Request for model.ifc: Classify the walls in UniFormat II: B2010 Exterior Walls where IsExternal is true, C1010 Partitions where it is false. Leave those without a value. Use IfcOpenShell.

First a look at what the model holds.

```python
import ifcopenshell
import ifcopenshell.util.element

model = ifcopenshell.open("model.ifc")
print(model.schema)
print("classifications:", [c.Name for c in model.by_type("IfcClassification")])
values = [ifcopenshell.util.element.get_pset(e, "Pset_WallCommon", "IsExternal") for e in model.by_type("IfcWall")]
for value in (True, False, None):
    print("IsExternal", value, values.count(value))
```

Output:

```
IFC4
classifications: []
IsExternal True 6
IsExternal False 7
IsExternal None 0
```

```python
import ifcopenshell
import ifcopenshell.api.classification
import ifcopenshell.util.element

model = ifcopenshell.open("model.ifc")

system = ifcopenshell.api.classification.add_classification(model, classification="UniFormat II")

walls = model.by_type("IfcWall")
external = {e: ifcopenshell.util.element.get_pset(e, "Pset_WallCommon", "IsExternal") for e in walls}
for flag, code, name in ((True, "B2010", "Exterior Walls"), (False, "C1010", "Partitions")):
    products = [e for e in walls if external[e] is flag]
    ifcopenshell.api.classification.add_reference(
        model, products=products, classification=system, identification=code, name=name
    )
    print(code, len(products))

model.write("model_updated.ifc")
```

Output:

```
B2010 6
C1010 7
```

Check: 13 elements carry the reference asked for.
